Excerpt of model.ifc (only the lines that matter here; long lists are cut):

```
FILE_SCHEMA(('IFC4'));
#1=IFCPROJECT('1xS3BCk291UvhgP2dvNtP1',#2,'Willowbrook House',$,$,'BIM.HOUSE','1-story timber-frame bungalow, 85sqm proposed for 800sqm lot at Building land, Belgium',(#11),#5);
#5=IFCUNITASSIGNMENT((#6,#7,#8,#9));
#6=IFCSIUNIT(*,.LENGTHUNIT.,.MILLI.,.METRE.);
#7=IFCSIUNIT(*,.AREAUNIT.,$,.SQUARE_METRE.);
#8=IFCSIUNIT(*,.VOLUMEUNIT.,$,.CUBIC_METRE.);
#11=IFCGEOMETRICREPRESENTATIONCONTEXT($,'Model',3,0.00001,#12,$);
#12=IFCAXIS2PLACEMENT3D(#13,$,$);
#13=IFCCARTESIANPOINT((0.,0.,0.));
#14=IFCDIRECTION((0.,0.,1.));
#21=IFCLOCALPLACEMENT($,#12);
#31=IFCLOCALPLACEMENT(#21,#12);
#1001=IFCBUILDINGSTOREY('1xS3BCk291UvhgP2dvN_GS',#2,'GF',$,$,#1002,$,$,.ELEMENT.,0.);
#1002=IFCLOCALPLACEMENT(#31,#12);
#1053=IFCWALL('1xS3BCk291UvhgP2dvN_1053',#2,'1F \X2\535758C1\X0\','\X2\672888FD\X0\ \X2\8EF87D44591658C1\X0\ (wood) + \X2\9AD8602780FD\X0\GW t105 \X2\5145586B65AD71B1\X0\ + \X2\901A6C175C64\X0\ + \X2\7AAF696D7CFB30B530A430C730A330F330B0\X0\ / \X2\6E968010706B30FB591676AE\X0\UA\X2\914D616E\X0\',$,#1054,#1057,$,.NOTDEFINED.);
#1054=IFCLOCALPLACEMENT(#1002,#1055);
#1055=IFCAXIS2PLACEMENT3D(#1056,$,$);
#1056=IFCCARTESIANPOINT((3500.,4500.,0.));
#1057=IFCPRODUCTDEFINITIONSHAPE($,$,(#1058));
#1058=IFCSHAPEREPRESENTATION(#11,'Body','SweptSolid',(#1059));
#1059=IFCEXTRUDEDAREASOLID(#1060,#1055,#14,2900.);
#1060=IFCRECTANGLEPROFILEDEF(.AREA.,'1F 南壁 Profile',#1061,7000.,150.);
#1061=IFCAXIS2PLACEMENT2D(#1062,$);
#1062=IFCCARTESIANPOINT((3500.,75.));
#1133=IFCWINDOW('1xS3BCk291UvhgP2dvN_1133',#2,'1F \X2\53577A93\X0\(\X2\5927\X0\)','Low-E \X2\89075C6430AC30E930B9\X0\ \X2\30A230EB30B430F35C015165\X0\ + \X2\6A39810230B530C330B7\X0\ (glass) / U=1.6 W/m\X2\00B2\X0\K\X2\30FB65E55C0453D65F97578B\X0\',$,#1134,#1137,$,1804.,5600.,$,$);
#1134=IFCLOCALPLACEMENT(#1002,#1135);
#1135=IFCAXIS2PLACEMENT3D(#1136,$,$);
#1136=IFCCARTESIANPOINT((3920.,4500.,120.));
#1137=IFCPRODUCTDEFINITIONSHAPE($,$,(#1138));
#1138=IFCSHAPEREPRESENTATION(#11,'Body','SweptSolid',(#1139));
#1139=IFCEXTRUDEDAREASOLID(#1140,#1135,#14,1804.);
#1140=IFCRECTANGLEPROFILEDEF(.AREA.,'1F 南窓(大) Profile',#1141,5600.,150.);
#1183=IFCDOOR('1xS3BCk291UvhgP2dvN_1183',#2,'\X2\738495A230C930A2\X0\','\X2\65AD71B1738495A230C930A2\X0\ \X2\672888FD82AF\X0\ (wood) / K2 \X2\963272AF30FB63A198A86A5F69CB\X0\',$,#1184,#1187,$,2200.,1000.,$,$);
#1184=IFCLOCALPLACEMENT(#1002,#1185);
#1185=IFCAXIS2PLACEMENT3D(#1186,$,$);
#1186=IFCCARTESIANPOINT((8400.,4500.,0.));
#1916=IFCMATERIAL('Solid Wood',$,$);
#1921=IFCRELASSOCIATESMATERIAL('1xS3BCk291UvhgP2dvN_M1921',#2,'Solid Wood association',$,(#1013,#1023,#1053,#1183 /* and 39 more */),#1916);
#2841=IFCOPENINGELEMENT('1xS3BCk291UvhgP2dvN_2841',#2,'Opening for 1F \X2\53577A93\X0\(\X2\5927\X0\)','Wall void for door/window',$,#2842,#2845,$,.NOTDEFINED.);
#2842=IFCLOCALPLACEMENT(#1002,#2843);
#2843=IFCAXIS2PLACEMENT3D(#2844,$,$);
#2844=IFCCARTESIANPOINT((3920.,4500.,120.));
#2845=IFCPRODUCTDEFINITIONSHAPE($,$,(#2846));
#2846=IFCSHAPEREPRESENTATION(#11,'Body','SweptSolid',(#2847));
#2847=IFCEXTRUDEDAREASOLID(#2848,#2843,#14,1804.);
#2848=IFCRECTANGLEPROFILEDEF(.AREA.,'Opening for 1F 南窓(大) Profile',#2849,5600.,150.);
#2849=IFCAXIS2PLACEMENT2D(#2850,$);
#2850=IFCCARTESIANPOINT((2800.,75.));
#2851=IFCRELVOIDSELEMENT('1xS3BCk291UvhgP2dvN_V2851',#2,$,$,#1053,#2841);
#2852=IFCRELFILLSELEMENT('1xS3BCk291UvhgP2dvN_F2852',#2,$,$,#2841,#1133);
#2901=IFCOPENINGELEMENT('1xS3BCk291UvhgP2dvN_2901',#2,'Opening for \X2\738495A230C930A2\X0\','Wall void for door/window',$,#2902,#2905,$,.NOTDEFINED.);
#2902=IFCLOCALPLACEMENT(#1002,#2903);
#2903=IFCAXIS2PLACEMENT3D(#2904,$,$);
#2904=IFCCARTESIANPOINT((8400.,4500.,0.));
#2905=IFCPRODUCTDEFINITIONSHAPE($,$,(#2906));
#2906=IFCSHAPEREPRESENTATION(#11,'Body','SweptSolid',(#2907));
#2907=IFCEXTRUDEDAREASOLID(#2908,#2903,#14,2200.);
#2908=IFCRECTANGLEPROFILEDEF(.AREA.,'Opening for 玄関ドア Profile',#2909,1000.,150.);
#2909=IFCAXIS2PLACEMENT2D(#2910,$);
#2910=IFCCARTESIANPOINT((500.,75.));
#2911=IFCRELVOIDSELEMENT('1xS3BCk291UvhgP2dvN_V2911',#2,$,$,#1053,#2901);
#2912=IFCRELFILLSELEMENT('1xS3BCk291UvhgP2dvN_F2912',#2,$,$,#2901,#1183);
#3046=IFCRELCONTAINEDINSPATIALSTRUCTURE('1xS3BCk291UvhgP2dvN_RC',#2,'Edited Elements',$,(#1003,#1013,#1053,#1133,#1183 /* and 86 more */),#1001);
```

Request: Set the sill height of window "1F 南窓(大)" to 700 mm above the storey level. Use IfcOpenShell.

```python
import numpy as np
import ifcopenshell
import ifcopenshell.api.geometry
import ifcopenshell.geom
import ifcopenshell.util.element
import ifcopenshell.util.placement
import ifcopenshell.util.shape
import ifcopenshell.util.unit

model = ifcopenshell.open("model.ifc")
unit_scale = ifcopenshell.util.unit.calculate_unit_scale(model)

window = model.by_guid("1xS3BCk291UvhgP2dvN_1133")
opening = window.FillsVoids[0].RelatingOpeningElement
storey = ifcopenshell.util.element.get_container(window, ifc_class="IfcBuildingStorey")
level = ifcopenshell.util.placement.get_local_placement(storey.ObjectPlacement)[2, 3]

# The opening's origin need not be at the sill, so measure its lowest point.
shape = ifcopenshell.geom.create_shape(ifcopenshell.geom.settings(), opening)
bottom = ifcopenshell.util.shape.get_shape_bottom_elevation(shape, shape.geometry) / unit_scale
dz = level + 700.0 - bottom

shift = np.array([0.0, 0.0, dz])
# The window is not placed relative to its opening, so move both.
for product in (opening, window):
    matrix = ifcopenshell.util.placement.get_local_placement(product.ObjectPlacement)
    matrix[:3, 3] += shift
    ifcopenshell.api.geometry.edit_object_placement(model, product=product, matrix=matrix, is_si=False)

print(f"moved by {dz * unit_scale:+.3f} m")

model.write("model_edited.ifc")
```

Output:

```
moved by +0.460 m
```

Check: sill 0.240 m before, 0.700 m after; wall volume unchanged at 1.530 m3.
